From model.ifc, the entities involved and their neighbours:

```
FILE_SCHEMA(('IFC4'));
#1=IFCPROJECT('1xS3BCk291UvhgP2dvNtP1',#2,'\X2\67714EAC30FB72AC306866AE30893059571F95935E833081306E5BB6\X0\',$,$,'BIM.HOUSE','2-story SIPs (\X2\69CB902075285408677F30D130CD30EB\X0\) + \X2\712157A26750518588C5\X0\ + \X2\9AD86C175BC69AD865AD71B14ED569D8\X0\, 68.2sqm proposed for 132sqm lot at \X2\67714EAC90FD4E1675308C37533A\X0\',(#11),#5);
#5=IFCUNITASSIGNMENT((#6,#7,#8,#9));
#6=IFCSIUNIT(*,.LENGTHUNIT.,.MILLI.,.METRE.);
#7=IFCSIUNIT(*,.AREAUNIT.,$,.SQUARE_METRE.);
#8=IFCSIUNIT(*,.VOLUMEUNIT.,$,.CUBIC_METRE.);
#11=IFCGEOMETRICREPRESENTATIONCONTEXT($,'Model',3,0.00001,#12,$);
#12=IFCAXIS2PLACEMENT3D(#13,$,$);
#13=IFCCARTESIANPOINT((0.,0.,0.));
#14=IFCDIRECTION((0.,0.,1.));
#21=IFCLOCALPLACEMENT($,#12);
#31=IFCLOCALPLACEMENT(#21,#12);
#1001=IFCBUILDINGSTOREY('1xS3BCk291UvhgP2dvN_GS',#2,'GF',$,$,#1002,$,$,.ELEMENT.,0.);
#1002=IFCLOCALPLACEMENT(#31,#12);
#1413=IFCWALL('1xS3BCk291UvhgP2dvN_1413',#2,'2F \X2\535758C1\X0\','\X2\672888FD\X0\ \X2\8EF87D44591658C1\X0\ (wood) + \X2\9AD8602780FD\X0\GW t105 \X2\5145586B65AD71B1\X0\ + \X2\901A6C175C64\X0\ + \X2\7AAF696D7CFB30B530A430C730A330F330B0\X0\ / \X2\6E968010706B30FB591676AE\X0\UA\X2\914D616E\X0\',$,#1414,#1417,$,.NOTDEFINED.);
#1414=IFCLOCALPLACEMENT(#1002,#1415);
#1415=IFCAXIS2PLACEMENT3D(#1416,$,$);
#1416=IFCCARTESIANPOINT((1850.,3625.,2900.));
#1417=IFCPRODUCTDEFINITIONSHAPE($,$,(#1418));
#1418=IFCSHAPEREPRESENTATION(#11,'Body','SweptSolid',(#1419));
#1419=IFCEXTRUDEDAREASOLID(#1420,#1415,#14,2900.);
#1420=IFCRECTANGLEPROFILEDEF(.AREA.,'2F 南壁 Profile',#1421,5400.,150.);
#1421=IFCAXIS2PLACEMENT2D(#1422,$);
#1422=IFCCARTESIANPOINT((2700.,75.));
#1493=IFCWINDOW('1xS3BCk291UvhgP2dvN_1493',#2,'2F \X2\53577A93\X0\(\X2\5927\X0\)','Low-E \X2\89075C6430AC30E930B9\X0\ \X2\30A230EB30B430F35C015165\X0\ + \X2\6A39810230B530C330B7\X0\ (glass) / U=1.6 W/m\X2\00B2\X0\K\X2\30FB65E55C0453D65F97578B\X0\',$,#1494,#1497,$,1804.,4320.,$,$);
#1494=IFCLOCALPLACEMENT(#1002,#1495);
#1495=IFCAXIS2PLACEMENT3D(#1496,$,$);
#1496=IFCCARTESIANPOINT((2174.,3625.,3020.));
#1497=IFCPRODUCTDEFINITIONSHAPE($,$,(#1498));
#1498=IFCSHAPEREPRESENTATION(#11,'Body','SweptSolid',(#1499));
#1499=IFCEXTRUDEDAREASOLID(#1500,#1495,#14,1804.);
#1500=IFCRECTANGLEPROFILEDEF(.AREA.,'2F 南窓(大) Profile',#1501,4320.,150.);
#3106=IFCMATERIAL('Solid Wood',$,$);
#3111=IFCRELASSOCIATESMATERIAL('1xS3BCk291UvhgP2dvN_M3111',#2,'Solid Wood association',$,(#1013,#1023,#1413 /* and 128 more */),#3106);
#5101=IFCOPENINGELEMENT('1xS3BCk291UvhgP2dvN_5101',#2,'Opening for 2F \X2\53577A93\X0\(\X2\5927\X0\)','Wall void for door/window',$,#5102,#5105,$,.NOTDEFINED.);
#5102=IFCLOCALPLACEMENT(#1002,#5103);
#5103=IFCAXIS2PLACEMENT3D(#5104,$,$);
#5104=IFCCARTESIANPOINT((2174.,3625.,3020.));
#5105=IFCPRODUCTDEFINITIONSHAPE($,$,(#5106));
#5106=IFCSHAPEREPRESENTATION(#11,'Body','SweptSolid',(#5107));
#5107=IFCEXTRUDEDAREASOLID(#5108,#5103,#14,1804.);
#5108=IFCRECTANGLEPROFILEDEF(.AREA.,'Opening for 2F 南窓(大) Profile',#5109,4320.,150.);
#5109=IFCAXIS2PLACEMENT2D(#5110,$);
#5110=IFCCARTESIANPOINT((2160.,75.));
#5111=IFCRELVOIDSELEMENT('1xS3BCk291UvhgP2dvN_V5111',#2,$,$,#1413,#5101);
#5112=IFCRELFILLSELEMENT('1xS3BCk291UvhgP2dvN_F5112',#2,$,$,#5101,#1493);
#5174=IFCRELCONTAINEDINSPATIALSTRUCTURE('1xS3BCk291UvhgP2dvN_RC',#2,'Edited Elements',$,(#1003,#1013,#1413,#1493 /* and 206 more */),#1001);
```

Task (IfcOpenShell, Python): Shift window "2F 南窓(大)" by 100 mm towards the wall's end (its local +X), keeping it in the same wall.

```python
import ifcopenshell
import ifcopenshell.api.geometry
import ifcopenshell.util.placement
import ifcopenshell.util.unit

model = ifcopenshell.open("model.ifc")
unit_scale = ifcopenshell.util.unit.calculate_unit_scale(model)

window = model.by_guid("1xS3BCk291UvhgP2dvN_1493")
opening = window.FillsVoids[0].RelatingOpeningElement
wall = opening.VoidsElements[0].RelatingBuildingElement

wall_matrix = ifcopenshell.util.placement.get_local_placement(wall.ObjectPlacement)
shift = wall_matrix[:3, 0] * 0.1 / unit_scale
before = ifcopenshell.util.placement.get_local_placement(window.ObjectPlacement)[:3, 3].copy()

# The window is not placed relative to its opening, so move both.
for product in (opening, window):
    matrix = ifcopenshell.util.placement.get_local_placement(product.ObjectPlacement)
    matrix[:3, 3] += shift
    ifcopenshell.api.geometry.edit_object_placement(model, product=product, matrix=matrix, is_si=False)

after = ifcopenshell.util.placement.get_local_placement(window.ObjectPlacement)[:3, 3]
print("window moved by", (after - before).round(3) + 0.0)

model.write("model-out.ifc")
```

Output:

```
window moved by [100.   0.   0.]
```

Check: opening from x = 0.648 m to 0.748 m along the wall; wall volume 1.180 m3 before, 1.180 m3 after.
